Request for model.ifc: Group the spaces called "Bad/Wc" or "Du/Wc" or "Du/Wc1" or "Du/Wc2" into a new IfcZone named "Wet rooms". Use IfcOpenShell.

First a look at what the model holds.

```python
import ifcopenshell

model = ifcopenshell.open("model.ifc")
print(model.schema)
seen = {}
for space in model.by_type("IfcSpace"):
    seen[space.LongName] = seen.get(space.LongName, 0) + 1
for name, count in sorted(seen.items(), key=str):
    print(count, "x", name)
print("zones:", [z.Name for z in model.by_type("IfcZone")][:20])
```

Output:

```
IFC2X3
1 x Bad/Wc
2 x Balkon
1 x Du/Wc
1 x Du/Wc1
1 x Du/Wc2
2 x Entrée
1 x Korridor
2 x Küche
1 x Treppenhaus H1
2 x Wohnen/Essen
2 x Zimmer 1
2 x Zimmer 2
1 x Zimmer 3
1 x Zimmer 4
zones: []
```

```python
import ifcopenshell
import ifcopenshell.api.group
import ifcopenshell.api.root

model = ifcopenshell.open("model.ifc")

names = {"Bad/Wc", "Du/Wc", "Du/Wc1", "Du/Wc2"}
spaces = [s for s in model.by_type("IfcSpace") if s.LongName in names]

zone = ifcopenshell.api.root.create_entity(model, ifc_class="IfcZone", name="Wet rooms")
ifcopenshell.api.group.assign_group(model, products=spaces, group=zone)
print(len(spaces), "spaces in", zone.Name)

model.write("model_updated.ifc")
```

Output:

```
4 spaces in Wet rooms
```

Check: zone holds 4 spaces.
